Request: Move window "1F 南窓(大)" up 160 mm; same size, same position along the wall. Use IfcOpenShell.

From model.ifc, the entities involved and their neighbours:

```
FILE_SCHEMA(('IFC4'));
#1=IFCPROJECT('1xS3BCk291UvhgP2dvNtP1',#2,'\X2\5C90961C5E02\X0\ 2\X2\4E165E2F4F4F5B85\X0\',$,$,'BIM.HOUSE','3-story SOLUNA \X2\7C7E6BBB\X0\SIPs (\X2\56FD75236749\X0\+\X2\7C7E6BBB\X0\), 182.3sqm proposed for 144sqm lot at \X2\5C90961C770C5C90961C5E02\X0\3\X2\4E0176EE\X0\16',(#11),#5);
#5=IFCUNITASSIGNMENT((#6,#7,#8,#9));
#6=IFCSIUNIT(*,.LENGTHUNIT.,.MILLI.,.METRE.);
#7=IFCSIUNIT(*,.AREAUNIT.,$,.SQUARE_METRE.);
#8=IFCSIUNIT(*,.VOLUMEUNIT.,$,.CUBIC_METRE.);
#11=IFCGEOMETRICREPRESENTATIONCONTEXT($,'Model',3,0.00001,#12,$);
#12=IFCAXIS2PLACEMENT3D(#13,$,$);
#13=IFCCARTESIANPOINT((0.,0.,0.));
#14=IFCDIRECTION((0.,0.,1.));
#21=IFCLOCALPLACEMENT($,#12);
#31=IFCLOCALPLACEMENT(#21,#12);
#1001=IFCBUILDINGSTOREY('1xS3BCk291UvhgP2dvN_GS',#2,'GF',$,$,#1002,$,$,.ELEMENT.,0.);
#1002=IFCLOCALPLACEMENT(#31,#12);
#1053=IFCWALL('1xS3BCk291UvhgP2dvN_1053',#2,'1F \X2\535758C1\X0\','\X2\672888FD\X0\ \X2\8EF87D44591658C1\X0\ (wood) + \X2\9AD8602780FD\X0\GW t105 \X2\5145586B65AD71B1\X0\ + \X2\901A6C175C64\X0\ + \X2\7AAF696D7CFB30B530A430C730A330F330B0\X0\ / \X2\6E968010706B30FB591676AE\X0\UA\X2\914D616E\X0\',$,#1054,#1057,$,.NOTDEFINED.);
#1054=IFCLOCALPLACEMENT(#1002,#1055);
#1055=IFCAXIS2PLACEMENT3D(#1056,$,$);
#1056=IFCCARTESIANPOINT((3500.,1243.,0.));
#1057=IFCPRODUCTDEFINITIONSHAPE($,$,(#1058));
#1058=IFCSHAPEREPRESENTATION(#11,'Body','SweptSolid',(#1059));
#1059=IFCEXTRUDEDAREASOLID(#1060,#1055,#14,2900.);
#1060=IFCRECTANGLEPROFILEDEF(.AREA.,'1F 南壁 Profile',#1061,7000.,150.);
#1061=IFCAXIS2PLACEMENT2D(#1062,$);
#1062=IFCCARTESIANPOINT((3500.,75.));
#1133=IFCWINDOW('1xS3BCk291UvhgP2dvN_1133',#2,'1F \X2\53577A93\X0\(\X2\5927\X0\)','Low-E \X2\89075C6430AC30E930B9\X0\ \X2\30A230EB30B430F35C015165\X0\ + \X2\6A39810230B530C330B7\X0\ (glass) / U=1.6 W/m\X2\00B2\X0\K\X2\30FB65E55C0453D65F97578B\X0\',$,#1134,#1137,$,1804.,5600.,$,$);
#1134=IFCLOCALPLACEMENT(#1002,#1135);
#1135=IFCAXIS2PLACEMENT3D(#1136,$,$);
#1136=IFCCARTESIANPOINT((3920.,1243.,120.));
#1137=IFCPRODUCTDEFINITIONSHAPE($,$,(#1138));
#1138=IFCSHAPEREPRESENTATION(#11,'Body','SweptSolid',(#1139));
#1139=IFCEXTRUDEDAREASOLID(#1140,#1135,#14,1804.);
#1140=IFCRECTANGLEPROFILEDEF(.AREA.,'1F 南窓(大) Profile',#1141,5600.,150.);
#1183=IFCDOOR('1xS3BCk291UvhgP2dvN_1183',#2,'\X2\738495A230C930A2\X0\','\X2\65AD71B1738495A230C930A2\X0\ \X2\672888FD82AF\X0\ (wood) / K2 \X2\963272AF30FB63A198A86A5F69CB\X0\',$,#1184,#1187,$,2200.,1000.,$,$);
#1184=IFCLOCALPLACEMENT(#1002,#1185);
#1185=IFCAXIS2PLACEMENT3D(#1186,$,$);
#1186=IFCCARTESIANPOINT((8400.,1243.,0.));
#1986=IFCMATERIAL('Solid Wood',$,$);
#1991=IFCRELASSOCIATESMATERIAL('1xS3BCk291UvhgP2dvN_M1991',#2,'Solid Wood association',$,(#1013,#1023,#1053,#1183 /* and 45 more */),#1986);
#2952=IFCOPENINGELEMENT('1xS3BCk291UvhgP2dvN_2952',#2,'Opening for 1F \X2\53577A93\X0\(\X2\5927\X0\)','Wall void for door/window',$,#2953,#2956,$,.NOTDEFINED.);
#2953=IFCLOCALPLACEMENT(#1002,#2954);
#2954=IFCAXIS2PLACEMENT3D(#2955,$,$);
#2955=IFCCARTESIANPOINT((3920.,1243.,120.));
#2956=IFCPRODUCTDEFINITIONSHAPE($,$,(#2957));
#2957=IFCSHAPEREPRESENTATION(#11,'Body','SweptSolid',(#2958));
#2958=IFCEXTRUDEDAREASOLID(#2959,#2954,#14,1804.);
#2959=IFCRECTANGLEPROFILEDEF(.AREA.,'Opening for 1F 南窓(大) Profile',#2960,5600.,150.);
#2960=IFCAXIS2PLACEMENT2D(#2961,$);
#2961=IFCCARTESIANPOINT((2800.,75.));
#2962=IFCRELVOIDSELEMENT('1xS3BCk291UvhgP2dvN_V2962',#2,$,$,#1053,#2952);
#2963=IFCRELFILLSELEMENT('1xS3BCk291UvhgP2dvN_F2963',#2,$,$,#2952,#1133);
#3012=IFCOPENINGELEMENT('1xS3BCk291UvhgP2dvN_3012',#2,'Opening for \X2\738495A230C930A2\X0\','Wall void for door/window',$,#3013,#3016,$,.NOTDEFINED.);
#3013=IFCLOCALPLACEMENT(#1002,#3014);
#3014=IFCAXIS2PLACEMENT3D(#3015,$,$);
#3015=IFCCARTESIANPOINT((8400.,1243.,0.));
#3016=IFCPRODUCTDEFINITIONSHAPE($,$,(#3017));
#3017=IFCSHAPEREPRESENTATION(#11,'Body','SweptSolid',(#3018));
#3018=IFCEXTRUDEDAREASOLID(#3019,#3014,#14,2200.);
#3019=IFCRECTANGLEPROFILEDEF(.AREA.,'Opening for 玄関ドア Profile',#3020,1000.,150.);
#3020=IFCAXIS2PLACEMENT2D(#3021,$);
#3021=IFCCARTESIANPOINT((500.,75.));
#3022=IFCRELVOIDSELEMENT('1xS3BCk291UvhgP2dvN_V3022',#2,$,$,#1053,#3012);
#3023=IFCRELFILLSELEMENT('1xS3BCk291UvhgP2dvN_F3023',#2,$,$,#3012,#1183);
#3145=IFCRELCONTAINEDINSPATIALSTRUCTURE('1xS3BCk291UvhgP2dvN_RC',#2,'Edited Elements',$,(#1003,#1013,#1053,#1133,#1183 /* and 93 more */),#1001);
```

```python
import numpy as np
import ifcopenshell
import ifcopenshell.api.geometry
import ifcopenshell.util.placement
import ifcopenshell.util.unit

model = ifcopenshell.open("model.ifc")
unit_scale = ifcopenshell.util.unit.calculate_unit_scale(model)

window = model.by_guid("1xS3BCk291UvhgP2dvN_1133")
opening = window.FillsVoids[0].RelatingOpeningElement
dz = 160.0

shift = np.array([0.0, 0.0, dz])
# The window is not placed relative to its opening, so move both.
for product in (opening, window):
    matrix = ifcopenshell.util.placement.get_local_placement(product.ObjectPlacement)
    matrix[:3, 3] += shift
    ifcopenshell.api.geometry.edit_object_placement(model, product=product, matrix=matrix, is_si=False)

print(f"moved by {dz * unit_scale:+.3f} m")

model.write("model_updated.ifc")
```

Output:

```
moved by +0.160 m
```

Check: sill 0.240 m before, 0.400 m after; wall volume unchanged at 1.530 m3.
